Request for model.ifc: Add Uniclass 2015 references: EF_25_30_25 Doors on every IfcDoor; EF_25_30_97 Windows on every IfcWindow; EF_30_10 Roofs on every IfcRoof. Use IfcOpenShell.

First a look at what the model holds.

```python
import ifcopenshell

model = ifcopenshell.open("model.ifc")
print(model.schema)
print("classifications:", [c.Name for c in model.by_type("IfcClassification")])
for ifc_class in ("IfcDoor", "IfcRoof", "IfcStair", "IfcWall", "IfcWindow"):
    print(ifc_class, len(model.by_type(ifc_class)))
```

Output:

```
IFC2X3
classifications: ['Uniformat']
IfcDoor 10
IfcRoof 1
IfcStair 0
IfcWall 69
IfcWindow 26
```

```python
import ifcopenshell
import ifcopenshell.api.classification

model = ifcopenshell.open("model.ifc")

# IFC2X3 requires Source and Edition and has no link from the project to the system.
system = model.create_entity("IfcClassification", Source="NBS", Edition="2015", Name="Uniclass 2015")

codes = {
    "IfcDoor": ("EF_25_30_25", "Doors"),
    "IfcWindow": ("EF_25_30_97", "Windows"),
    "IfcRoof": ("EF_30_10", "Roofs"),
}
for ifc_class, (code, name) in codes.items():
    products = model.by_type(ifc_class)
    ifcopenshell.api.classification.add_reference(
        model, products=products, classification=system, identification=code, name=name
    )
    print(code, len(products))

model.write("model_v2.ifc")
```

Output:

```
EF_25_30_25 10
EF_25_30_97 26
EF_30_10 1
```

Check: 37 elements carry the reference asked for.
